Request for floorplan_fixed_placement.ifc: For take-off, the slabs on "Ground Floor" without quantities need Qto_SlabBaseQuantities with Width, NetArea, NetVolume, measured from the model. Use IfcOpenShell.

First a look at what the model holds.

```python
import ifcopenshell
import ifcopenshell.util.element
import ifcopenshell.util.unit

model = ifcopenshell.open("floorplan_fixed_placement.ifc")
print(model.schema)
for unit_type in ("LENGTHUNIT", "AREAUNIT", "VOLUMEUNIT"):
    print(unit_type, ifcopenshell.util.unit.calculate_unit_scale(model, unit_type))
storey = next(s for s in model.by_type("IfcBuildingStorey") if s.Name == "Ground Floor")
slabs = [e for e in ifcopenshell.util.element.get_decomposition(storey) if e.is_a("IfcSlab")]
for e in sorted(slabs, key=lambda e: e.id()):
    print(e.id(), e.is_a(), e.Name, list(ifcopenshell.util.element.get_psets(e, qtos_only=True)), sep=" | ")
```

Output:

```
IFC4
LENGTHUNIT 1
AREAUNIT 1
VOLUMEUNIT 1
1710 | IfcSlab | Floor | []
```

```python
import ifcopenshell
import ifcopenshell.api.pset
import ifcopenshell.geom
import ifcopenshell.util.element
import ifcopenshell.util.shape
import ifcopenshell.util.unit

model = ifcopenshell.open("floorplan_fixed_placement.ifc")
unit_scale = ifcopenshell.util.unit.calculate_unit_scale(model)
area_scale = ifcopenshell.util.unit.calculate_unit_scale(model, "AREAUNIT")
volume_scale = ifcopenshell.util.unit.calculate_unit_scale(model, "VOLUMEUNIT")
settings = ifcopenshell.geom.settings()

storey = next(s for s in model.by_type("IfcBuildingStorey") if s.Name == "Ground Floor")
slabs = [e for e in ifcopenshell.util.element.get_decomposition(storey) if e.is_a("IfcSlab")]

for e in sorted(slabs, key=lambda e: e.id()):
    if ifcopenshell.util.element.get_psets(e, qtos_only=True, should_inherit=False):
        continue
    # Geometry comes back in metres, in the element's own axes.
    shape = ifcopenshell.geom.create_shape(settings, e)
    values = {
        "Width": ifcopenshell.util.shape.get_z(shape.geometry) / unit_scale,
        "NetArea": ifcopenshell.util.shape.get_footprint_area(shape.geometry) / area_scale,
        "NetVolume": ifcopenshell.util.shape.get_volume(shape.geometry) / volume_scale,
    }
    qto = ifcopenshell.api.pset.add_qto(model, product=e, name="Qto_SlabBaseQuantities")
    ifcopenshell.api.pset.edit_qto(model, qto=qto, properties=values)
    print(e.id(), {k: round(v, 3) for k, v in values.items()})

model.write("floorplan_fixed_placement_updated.ifc")
```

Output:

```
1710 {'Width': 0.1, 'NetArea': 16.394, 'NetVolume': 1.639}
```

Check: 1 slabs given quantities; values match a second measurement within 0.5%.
